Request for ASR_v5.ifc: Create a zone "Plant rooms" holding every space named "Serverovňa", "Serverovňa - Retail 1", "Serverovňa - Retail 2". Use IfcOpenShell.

First a look at what the model holds.

```python
import ifcopenshell

model = ifcopenshell.open("ASR_v5.ifc")
print(model.schema)
seen = {}
for space in model.by_type("IfcSpace"):
    seen[space.LongName] = seen.get(space.LongName, 0) + 1
for name, count in sorted(seen.items(), key=str):
    print(count, "x", name)
print("zones:", [z.Name for z in model.by_type("IfcZone")][:20])
```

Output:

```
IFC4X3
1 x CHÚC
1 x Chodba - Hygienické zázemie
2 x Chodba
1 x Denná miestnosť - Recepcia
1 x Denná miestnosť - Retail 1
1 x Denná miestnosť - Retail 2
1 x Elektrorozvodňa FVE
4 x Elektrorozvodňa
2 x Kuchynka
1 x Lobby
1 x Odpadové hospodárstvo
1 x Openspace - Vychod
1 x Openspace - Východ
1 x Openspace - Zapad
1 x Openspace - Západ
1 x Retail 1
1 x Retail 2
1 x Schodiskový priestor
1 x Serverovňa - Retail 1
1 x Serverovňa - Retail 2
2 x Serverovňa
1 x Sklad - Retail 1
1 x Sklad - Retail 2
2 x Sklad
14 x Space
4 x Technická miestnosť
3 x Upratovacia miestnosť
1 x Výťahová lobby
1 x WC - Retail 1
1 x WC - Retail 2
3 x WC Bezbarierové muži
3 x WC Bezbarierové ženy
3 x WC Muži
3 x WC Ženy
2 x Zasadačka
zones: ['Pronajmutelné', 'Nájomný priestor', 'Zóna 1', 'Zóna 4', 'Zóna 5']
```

```python
import ifcopenshell
import ifcopenshell.api.group
import ifcopenshell.api.root

model = ifcopenshell.open("ASR_v5.ifc")

names = {"Serverovňa", "Serverovňa - Retail 1", "Serverovňa - Retail 2"}
spaces = [s for s in model.by_type("IfcSpace") if s.LongName in names]

zone = ifcopenshell.api.root.create_entity(model, ifc_class="IfcZone", name="Plant rooms")
ifcopenshell.api.group.assign_group(model, products=spaces, group=zone)
print(len(spaces), "spaces in", zone.Name)

model.write("ASR_v5_rev.ifc")
```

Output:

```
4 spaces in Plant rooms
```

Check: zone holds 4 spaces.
